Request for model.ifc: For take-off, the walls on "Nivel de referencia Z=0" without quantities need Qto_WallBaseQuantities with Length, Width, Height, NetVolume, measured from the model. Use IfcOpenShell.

First a look at what the model holds.

```python
import ifcopenshell
import ifcopenshell.util.element
import ifcopenshell.util.unit

model = ifcopenshell.open("model.ifc")
print(model.schema)
for unit_type in ("LENGTHUNIT", "AREAUNIT", "VOLUMEUNIT"):
    print(unit_type, ifcopenshell.util.unit.calculate_unit_scale(model, unit_type))
storey = next(s for s in model.by_type("IfcBuildingStorey") if s.Name == "Nivel de referencia Z=0")
walls = [e for e in ifcopenshell.util.element.get_decomposition(storey) if e.is_a("IfcWall")]
for e in sorted(walls, key=lambda e: e.id()):
    print(e.id(), e.is_a(), e.Name, list(ifcopenshell.util.element.get_psets(e, qtos_only=True)), sep=" | ")
```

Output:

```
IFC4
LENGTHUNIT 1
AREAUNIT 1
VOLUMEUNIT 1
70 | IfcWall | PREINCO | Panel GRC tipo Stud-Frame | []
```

```python
import ifcopenshell
import ifcopenshell.api.pset
import ifcopenshell.geom
import ifcopenshell.util.element
import ifcopenshell.util.shape
import ifcopenshell.util.unit

model = ifcopenshell.open("model.ifc")
unit_scale = ifcopenshell.util.unit.calculate_unit_scale(model)
volume_scale = ifcopenshell.util.unit.calculate_unit_scale(model, "VOLUMEUNIT")
settings = ifcopenshell.geom.settings()

storey = next(s for s in model.by_type("IfcBuildingStorey") if s.Name == "Nivel de referencia Z=0")
walls = [e for e in ifcopenshell.util.element.get_decomposition(storey) if e.is_a("IfcWall")]

for e in sorted(walls, key=lambda e: e.id()):
    if ifcopenshell.util.element.get_psets(e, qtos_only=True, should_inherit=False):
        continue
    # Geometry comes back in metres, in the element's own axes.
    shape = ifcopenshell.geom.create_shape(settings, e)
    values = {
        "Length": ifcopenshell.util.shape.get_x(shape.geometry) / unit_scale,
        "Width": ifcopenshell.util.shape.get_y(shape.geometry) / unit_scale,
        "Height": ifcopenshell.util.shape.get_z(shape.geometry) / unit_scale,
        "NetVolume": ifcopenshell.util.shape.get_volume(shape.geometry) / volume_scale,
    }
    qto = ifcopenshell.api.pset.add_qto(model, product=e, name="Qto_WallBaseQuantities")
    ifcopenshell.api.pset.edit_qto(model, qto=qto, properties=values)
    print(e.id(), {k: round(v, 3) for k, v in values.items()})

model.write("model_updated.ifc")
```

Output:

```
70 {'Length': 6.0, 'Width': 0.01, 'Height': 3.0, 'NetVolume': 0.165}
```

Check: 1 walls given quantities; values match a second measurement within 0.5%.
